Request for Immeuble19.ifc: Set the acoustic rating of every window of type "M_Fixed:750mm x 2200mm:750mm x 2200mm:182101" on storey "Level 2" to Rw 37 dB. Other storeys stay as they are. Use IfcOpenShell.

First a look at what the model holds.

```python
import ifcopenshell
import ifcopenshell.util.element

model = ifcopenshell.open("Immeuble19.ifc")
print(model.schema)
storey = next(s for s in model.by_type("IfcBuildingStorey") if s.Name == "Level 2")
windows = [e for e in ifcopenshell.util.element.get_decomposition(storey) if e.is_a("IfcWindow")]
seen = {}
for e in windows:
    element_type = ifcopenshell.util.element.get_type(e)
    key = (element_type.Name if element_type != e and element_type else None, ifcopenshell.util.element.get_pset(e, "Pset_WindowCommon", "AcousticRating"))
    seen[key] = seen.get(key, 0) + 1
for (name, value), count in sorted(seen.items(), key=str):
    print(count, "x", name, "|", value)
```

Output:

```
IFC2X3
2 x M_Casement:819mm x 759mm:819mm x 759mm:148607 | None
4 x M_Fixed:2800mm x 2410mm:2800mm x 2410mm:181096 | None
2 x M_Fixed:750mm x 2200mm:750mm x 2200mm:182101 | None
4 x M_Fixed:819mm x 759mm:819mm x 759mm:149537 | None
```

```python
import ifcopenshell
import ifcopenshell.api.pset
import ifcopenshell.util.element

model = ifcopenshell.open("Immeuble19.ifc")

storey = next(s for s in model.by_type("IfcBuildingStorey") if s.Name == "Level 2")
windows = [e for e in ifcopenshell.util.element.get_decomposition(storey) if e.is_a("IfcWindow")]

count = 0
for e in windows:
    element_type = ifcopenshell.util.element.get_type(e)
    if element_type in (None, e) or element_type.Name != "M_Fixed:750mm x 2200mm:750mm x 2200mm:182101":
        continue
    # add_pset returns the element's existing set when there is one.
    pset = ifcopenshell.api.pset.add_pset(model, product=e, name="Pset_WindowCommon")
    ifcopenshell.api.pset.edit_pset(model, pset=pset, properties={"AcousticRating": "Rw 37 dB"})
    count += 1

print(count, "windows updated")

model.write("Immeuble19_rev.ifc")
```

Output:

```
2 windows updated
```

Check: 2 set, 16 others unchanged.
